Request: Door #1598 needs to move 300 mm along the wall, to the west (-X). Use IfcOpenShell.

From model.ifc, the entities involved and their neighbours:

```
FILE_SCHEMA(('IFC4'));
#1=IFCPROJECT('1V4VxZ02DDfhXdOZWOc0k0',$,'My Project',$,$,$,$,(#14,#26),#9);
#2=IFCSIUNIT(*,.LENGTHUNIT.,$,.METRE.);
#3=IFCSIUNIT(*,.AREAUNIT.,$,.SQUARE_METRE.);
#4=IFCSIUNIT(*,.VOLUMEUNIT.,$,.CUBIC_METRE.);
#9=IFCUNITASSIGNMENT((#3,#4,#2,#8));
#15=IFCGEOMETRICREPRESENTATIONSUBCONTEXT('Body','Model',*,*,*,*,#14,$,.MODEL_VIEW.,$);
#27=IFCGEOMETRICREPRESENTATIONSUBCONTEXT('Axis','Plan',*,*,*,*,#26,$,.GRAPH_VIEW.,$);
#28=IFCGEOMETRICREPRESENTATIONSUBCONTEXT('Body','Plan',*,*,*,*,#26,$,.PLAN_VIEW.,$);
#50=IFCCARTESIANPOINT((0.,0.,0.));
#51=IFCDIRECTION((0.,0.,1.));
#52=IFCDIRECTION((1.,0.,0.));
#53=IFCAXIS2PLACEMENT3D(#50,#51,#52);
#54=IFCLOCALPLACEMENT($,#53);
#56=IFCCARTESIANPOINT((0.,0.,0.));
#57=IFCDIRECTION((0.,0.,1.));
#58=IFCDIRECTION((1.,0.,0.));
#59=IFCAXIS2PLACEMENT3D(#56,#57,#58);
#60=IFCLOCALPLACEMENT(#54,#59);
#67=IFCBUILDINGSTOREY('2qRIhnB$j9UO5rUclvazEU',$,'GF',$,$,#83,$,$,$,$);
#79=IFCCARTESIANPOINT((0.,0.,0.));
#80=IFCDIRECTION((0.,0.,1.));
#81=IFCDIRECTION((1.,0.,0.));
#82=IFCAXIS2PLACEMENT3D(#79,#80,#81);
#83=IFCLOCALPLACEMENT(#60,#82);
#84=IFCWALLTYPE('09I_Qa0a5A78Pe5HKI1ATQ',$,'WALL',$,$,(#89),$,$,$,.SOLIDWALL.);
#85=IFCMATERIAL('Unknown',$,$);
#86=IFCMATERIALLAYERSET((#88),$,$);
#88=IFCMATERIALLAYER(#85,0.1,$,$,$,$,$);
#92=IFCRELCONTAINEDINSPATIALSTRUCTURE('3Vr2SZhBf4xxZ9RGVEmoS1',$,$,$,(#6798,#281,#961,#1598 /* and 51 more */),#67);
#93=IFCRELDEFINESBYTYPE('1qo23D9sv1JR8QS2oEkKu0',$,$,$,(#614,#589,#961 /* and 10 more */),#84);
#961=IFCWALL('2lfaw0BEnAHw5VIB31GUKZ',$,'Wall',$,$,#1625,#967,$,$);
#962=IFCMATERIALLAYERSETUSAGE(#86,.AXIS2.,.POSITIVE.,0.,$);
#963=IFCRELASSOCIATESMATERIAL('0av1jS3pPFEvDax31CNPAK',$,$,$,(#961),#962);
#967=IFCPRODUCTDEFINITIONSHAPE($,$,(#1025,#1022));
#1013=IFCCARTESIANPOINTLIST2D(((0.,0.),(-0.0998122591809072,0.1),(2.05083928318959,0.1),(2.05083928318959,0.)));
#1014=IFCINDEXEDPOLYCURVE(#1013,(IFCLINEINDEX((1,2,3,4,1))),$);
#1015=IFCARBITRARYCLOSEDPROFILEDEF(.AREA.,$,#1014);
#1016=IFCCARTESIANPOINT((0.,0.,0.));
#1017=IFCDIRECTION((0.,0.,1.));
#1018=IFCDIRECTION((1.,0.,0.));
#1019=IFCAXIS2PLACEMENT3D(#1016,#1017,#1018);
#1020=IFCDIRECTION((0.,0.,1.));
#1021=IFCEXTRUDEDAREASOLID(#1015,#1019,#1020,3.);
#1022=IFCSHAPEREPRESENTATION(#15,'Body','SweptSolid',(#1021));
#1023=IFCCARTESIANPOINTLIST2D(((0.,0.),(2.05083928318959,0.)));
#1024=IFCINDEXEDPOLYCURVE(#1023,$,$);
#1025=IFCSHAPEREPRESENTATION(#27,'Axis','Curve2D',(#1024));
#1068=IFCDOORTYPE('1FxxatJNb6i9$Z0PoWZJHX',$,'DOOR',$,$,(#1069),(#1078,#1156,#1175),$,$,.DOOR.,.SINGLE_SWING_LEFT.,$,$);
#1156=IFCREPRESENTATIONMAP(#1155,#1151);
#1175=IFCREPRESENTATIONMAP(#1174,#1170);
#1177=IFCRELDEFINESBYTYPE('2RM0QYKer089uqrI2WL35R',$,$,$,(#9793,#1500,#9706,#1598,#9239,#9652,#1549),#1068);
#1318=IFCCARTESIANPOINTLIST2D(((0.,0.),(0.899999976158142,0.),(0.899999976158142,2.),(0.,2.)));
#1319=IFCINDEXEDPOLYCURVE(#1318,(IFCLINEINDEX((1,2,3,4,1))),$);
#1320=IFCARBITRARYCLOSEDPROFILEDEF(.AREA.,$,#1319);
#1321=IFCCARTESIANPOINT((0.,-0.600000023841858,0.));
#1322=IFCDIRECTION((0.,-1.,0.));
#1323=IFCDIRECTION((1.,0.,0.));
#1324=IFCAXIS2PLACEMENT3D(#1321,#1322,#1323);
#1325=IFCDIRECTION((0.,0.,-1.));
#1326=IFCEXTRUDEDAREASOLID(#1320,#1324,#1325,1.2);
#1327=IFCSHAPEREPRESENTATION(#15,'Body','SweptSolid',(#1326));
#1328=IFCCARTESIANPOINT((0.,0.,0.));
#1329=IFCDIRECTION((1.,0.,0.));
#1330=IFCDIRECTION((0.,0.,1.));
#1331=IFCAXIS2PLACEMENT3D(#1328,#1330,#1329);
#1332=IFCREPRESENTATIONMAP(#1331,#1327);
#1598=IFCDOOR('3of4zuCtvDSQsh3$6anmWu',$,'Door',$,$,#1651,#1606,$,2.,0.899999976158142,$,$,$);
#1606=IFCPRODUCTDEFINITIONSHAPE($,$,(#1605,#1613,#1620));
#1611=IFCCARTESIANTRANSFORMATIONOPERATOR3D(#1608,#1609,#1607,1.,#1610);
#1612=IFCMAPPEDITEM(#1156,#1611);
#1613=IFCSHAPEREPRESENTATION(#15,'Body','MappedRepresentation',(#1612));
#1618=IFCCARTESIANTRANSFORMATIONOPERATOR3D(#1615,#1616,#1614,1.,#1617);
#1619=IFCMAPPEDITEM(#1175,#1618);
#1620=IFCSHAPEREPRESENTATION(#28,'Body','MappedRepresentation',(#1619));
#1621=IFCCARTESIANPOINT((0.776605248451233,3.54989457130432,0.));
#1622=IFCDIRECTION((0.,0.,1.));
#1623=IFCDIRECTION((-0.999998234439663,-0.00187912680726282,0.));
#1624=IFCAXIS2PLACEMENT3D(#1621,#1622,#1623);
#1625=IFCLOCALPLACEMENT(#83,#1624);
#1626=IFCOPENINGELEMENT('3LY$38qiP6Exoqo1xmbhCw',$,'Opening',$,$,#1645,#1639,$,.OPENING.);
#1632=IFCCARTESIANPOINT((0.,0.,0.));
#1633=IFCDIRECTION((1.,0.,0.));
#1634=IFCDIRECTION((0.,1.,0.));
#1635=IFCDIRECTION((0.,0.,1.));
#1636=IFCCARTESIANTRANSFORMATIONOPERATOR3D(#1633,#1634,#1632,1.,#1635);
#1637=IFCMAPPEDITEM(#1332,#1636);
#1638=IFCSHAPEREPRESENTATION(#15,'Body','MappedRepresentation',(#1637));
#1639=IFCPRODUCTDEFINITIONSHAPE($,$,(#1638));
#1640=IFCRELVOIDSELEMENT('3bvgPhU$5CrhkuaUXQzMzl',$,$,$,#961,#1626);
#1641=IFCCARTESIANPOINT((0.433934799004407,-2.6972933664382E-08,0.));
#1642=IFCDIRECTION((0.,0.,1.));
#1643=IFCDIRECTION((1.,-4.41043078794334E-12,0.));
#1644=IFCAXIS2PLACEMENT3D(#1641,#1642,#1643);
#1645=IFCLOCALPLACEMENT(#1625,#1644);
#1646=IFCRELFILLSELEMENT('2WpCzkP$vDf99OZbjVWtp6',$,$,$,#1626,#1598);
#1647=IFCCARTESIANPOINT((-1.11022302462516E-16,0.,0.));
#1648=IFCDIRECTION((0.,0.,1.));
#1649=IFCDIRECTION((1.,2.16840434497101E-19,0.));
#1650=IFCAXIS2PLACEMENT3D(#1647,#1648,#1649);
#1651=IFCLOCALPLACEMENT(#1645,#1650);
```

```python
import ifcopenshell
import ifcopenshell.api.geometry
import ifcopenshell.util.placement
import ifcopenshell.util.unit

model = ifcopenshell.open("model.ifc")
unit_scale = ifcopenshell.util.unit.calculate_unit_scale(model)

door = model.by_guid("3of4zuCtvDSQsh3$6anmWu")
opening = door.FillsVoids[0].RelatingOpeningElement
wall = opening.VoidsElements[0].RelatingBuildingElement

wall_matrix = ifcopenshell.util.placement.get_local_placement(wall.ObjectPlacement)
shift = wall_matrix[:3, 0] * 0.3 / unit_scale
before = ifcopenshell.util.placement.get_local_placement(door.ObjectPlacement)[:3, 3].copy()

# The door is placed relative to its opening, so it follows when the opening moves.
matrix = ifcopenshell.util.placement.get_local_placement(opening.ObjectPlacement)
matrix[:3, 3] += shift
ifcopenshell.api.geometry.edit_object_placement(
    model, product=opening, matrix=matrix, is_si=False, should_transform_children=True
)

after = ifcopenshell.util.placement.get_local_placement(door.ObjectPlacement)[:3, 3]
print("door moved by", (after - before).round(3) + 0.0)

model.write("model_v2.ifc")
```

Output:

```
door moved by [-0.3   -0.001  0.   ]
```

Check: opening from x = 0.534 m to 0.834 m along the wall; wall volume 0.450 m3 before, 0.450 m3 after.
